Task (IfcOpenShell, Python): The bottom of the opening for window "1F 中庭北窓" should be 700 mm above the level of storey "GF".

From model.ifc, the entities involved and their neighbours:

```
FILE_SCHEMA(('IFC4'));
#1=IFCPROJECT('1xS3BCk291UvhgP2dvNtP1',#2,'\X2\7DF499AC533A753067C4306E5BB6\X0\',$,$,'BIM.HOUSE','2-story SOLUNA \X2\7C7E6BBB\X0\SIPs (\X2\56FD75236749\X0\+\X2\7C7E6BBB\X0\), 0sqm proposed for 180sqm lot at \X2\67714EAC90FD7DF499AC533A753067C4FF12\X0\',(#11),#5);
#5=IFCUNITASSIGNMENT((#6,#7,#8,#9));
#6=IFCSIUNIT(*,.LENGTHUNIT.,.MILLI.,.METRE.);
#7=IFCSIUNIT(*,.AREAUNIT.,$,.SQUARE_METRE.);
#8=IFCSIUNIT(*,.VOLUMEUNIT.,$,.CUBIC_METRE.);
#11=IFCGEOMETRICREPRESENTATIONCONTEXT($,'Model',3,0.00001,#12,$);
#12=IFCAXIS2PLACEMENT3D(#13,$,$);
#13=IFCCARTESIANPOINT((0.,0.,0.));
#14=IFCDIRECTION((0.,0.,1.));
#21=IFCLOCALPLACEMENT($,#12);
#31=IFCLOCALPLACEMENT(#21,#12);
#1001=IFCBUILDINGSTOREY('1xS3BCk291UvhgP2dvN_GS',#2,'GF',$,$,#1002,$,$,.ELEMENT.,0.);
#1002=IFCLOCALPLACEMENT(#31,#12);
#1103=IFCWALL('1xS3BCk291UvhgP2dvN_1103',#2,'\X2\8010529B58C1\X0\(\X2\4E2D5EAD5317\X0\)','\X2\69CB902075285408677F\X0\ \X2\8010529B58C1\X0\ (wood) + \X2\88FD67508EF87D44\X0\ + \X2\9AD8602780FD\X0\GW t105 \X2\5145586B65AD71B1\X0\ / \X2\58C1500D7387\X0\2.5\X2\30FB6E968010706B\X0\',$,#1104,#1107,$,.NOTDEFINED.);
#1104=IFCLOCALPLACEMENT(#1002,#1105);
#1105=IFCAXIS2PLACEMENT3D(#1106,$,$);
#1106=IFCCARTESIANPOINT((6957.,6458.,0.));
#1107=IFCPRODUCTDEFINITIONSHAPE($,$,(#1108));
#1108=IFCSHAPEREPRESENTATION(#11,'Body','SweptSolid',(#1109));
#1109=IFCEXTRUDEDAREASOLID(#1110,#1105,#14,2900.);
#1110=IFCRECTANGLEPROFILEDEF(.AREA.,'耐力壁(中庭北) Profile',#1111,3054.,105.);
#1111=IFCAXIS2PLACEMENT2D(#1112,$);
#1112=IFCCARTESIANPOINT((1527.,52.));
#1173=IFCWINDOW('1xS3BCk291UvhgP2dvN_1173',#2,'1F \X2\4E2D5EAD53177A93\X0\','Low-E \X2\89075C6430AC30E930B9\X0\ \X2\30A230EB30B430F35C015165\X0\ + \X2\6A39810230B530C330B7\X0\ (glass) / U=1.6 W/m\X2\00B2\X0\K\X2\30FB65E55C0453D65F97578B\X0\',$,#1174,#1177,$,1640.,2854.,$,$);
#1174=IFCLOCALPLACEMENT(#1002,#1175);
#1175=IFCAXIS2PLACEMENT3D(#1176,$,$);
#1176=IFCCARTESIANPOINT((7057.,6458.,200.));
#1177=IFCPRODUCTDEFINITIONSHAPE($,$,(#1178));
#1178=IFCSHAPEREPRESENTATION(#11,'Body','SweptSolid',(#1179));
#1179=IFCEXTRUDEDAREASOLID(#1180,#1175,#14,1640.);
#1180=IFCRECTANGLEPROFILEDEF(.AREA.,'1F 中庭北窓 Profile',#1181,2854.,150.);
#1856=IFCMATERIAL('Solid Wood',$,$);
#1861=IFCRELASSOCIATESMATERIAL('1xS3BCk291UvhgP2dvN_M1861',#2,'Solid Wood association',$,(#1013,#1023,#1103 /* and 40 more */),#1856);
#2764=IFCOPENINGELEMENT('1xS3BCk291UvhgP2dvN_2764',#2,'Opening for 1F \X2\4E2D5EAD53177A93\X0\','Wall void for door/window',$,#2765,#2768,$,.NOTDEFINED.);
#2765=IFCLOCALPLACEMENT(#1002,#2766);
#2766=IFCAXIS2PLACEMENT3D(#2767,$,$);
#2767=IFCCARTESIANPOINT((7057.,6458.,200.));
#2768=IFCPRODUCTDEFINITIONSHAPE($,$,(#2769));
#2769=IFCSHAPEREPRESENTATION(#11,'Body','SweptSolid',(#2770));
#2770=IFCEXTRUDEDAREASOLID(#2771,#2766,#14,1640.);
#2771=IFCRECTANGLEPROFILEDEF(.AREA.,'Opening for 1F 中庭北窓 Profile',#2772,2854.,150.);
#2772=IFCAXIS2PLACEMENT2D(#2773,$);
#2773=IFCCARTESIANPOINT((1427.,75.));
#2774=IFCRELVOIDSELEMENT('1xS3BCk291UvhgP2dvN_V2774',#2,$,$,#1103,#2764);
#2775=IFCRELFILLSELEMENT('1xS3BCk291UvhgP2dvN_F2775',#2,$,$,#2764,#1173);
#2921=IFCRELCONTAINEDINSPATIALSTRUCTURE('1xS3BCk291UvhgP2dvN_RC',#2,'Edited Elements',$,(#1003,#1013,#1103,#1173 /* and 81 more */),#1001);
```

```python
import numpy as np
import ifcopenshell
import ifcopenshell.api.geometry
import ifcopenshell.geom
import ifcopenshell.util.element
import ifcopenshell.util.placement
import ifcopenshell.util.shape
import ifcopenshell.util.unit

model = ifcopenshell.open("model.ifc")
unit_scale = ifcopenshell.util.unit.calculate_unit_scale(model)

window = model.by_guid("1xS3BCk291UvhgP2dvN_1173")
opening = window.FillsVoids[0].RelatingOpeningElement
storey = ifcopenshell.util.element.get_container(window, ifc_class="IfcBuildingStorey")
level = ifcopenshell.util.placement.get_local_placement(storey.ObjectPlacement)[2, 3]

# The opening's origin need not be at the sill, so measure its lowest point.
shape = ifcopenshell.geom.create_shape(ifcopenshell.geom.settings(), opening)
bottom = ifcopenshell.util.shape.get_shape_bottom_elevation(shape, shape.geometry) / unit_scale
dz = level + 700.0 - bottom

shift = np.array([0.0, 0.0, dz])
# The window is not placed relative to its opening, so move both.
for product in (opening, window):
    matrix = ifcopenshell.util.placement.get_local_placement(product.ObjectPlacement)
    matrix[:3, 3] += shift
    ifcopenshell.api.geometry.edit_object_placement(model, product=product, matrix=matrix, is_si=False)

print(f"moved by {dz * unit_scale:+.3f} m")

model.write("model-out.ifc")
```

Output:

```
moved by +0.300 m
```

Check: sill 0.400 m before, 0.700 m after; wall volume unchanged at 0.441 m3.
